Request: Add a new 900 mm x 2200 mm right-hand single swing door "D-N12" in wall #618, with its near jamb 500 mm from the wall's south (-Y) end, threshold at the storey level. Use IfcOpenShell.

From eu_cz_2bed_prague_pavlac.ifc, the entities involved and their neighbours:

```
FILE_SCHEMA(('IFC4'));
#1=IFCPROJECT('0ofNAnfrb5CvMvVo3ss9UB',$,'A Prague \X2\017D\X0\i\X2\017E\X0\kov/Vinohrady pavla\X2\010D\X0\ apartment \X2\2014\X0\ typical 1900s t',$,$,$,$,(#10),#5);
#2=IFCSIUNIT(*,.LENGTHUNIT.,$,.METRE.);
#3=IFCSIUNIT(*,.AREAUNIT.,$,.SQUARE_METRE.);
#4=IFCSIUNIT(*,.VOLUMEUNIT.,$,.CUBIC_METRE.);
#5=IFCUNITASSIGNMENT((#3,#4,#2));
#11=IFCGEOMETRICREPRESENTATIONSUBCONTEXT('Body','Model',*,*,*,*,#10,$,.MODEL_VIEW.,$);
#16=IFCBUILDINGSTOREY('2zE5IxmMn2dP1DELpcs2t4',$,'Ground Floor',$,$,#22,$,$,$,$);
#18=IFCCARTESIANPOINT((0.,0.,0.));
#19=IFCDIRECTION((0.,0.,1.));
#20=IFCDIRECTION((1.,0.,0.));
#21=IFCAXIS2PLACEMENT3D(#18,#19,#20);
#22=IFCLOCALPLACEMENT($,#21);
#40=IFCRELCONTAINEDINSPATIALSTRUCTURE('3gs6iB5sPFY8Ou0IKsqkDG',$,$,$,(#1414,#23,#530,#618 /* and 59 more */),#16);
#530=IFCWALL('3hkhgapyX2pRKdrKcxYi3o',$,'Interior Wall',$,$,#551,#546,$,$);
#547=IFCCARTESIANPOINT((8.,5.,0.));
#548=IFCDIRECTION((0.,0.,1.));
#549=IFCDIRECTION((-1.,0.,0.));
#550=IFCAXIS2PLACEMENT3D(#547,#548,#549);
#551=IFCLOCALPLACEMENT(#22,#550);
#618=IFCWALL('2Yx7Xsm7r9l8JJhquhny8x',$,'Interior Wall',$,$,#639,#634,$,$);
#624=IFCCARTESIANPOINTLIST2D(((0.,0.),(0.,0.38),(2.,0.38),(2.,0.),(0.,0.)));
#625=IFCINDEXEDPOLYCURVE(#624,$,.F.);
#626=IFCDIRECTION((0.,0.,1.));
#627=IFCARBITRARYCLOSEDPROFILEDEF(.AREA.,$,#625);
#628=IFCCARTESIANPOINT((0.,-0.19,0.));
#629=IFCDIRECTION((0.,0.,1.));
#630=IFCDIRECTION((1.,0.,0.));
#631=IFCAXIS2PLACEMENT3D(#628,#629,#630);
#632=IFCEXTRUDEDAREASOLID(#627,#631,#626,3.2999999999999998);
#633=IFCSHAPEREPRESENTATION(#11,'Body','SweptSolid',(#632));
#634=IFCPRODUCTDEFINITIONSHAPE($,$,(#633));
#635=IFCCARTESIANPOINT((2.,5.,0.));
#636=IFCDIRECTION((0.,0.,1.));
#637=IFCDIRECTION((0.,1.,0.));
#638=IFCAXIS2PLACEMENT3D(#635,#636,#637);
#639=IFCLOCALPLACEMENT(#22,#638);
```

```python
import numpy as np
import ifcopenshell
import ifcopenshell.api.feature
import ifcopenshell.api.geometry
import ifcopenshell.api.root
import ifcopenshell.api.spatial
import ifcopenshell.geom
import ifcopenshell.util.element
import ifcopenshell.util.placement
import ifcopenshell.util.representation
import ifcopenshell.util.shape
import ifcopenshell.util.unit

model = ifcopenshell.open("eu_cz_2bed_prague_pavlac.ifc")
unit_scale = ifcopenshell.util.unit.calculate_unit_scale(model)
settings = ifcopenshell.geom.settings()


def volume(element):
    """Net volume in cubic metres, openings subtracted."""
    shape = ifcopenshell.geom.create_shape(settings, element)
    return ifcopenshell.util.shape.get_volume(shape.geometry)


wall = model.by_id(618)
storey = ifcopenshell.util.element.get_container(wall, ifc_class="IfcBuildingStorey")
context = ifcopenshell.util.representation.get_context(model, "Model", "Body", "MODEL_VIEW")
before = volume(wall)

width, height, from_end, sill = 0.9, 2.2, 0.5, 0.0  # metres

# The wall runs along its own X axis, and the end named is its -X end.
wall_shape = ifcopenshell.geom.create_shape(settings, wall)
x, y, z = ifcopenshell.util.shape.get_vertices(wall_shape.geometry).T
start = x.min() + from_end
face, thickness = float(y.min()), float(y.max() - y.min())
wall_matrix = ifcopenshell.util.placement.get_local_placement(wall.ObjectPlacement)
level = ifcopenshell.util.placement.get_local_placement(storey.ObjectPlacement)[2, 3]


def in_wall(x, y):
    """Placement at x, y metres in the wall's axes, at sill height."""
    matrix = wall_matrix.copy()
    matrix[:, 3] = wall_matrix @ np.array([x / unit_scale, y / unit_scale, 0.0, 1.0])
    matrix[2, 3] = level + sill / unit_scale
    return matrix


# Opening: a box that overshoots both wall faces by 50 mm.
opening = ifcopenshell.api.root.create_entity(model, ifc_class="IfcOpeningElement", predefined_type="OPENING")
box = ifcopenshell.api.geometry.add_wall_representation(
    model, context=context, length=width, height=height, thickness=thickness + 0.1
)
ifcopenshell.api.geometry.assign_representation(model, product=opening, representation=box)
ifcopenshell.api.geometry.edit_object_placement(model, product=opening, matrix=in_wall(start, face - 0.05), is_si=False)
ifcopenshell.api.feature.add_feature(model, feature=opening, element=wall)

door = ifcopenshell.api.root.create_entity(model, ifc_class="IfcDoor", name="D-N12", predefined_type="DOOR")
door.OverallWidth, door.OverallHeight = width / unit_scale, height / unit_scale
door.OperationType = "SINGLE_SWING_RIGHT"
body = ifcopenshell.api.geometry.add_door_representation(
    model,
    context=context,
    overall_width=door.OverallWidth,
    overall_height=door.OverallHeight,
    operation_type="SINGLE_SWING_RIGHT",
    lining_properties={"LiningDepth": thickness / unit_scale, "ThresholdDepth": thickness / unit_scale},
)
ifcopenshell.api.geometry.assign_representation(model, product=door, representation=body)
ifcopenshell.api.spatial.assign_container(model, products=[door], relating_structure=storey)
ifcopenshell.api.feature.add_filling(model, opening=opening, element=door)

# The lining spans the wall, so the door starts at the wall face.
ifcopenshell.api.geometry.edit_object_placement(model, product=door, matrix=in_wall(start, face), is_si=False)

after = volume(wall)

print(f"wall volume {before:.3f} -> {after:.3f} m3")

model.write("eu_cz_2bed_prague_pavlac_v2.ifc")
```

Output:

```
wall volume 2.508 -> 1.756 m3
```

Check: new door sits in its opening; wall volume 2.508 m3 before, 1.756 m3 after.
